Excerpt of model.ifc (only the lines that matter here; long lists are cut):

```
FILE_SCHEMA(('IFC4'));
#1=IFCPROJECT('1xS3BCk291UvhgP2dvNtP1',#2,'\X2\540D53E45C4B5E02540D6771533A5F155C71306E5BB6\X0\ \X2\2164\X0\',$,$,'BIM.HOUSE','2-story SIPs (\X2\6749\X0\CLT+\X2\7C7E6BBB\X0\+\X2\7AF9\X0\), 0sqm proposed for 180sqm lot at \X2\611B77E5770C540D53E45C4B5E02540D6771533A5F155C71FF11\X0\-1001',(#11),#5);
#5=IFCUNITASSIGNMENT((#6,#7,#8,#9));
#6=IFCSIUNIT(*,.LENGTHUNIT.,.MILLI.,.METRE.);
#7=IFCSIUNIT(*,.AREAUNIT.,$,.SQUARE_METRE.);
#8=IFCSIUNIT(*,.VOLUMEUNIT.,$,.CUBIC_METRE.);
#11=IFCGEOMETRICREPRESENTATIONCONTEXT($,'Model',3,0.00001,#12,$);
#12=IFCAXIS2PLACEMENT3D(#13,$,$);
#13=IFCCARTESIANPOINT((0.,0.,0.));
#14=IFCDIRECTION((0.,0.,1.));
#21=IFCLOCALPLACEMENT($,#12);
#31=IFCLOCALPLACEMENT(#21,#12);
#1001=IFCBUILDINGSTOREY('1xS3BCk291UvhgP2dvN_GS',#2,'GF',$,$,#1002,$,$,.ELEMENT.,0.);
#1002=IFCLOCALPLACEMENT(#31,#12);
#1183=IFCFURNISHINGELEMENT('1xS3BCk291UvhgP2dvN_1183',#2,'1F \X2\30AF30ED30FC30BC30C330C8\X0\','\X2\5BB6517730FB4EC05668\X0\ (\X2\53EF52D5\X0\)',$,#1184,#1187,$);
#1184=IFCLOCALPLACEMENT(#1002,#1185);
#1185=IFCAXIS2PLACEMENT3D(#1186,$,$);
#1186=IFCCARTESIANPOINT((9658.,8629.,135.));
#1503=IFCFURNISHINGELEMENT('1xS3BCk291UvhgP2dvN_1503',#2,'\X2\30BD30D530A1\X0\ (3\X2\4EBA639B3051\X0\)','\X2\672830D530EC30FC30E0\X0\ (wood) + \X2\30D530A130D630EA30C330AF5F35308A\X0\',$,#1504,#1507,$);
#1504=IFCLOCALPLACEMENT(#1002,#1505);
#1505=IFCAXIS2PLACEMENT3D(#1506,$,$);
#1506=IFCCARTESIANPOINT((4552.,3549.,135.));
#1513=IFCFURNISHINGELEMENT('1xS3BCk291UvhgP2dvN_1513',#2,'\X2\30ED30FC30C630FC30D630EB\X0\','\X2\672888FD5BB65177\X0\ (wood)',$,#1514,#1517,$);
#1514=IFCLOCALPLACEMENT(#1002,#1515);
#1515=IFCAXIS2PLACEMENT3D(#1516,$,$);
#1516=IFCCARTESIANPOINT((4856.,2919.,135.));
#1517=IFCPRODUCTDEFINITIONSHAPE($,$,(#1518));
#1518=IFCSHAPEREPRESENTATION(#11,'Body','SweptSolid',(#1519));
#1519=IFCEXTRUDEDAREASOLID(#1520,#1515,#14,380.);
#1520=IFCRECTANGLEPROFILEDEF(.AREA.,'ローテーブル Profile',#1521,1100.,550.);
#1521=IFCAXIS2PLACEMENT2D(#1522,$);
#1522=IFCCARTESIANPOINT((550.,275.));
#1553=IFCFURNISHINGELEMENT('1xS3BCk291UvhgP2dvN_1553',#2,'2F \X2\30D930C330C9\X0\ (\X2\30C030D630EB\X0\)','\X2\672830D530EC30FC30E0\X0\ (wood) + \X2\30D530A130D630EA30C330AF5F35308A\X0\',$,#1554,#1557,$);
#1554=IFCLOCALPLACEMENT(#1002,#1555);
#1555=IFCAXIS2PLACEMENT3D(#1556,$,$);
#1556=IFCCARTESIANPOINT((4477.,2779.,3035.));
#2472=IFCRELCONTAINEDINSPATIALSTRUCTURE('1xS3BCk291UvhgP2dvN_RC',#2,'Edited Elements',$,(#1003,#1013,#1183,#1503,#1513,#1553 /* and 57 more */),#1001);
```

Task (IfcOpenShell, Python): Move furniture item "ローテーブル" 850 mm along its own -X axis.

```python
import ifcopenshell
import ifcopenshell.api.geometry
import ifcopenshell.util.placement
import ifcopenshell.util.unit

model = ifcopenshell.open("model.ifc")
unit_scale = ifcopenshell.util.unit.calculate_unit_scale(model)

item = model.by_guid("1xS3BCk291UvhgP2dvN_1513")
matrix = ifcopenshell.util.placement.get_local_placement(item.ObjectPlacement)
matrix[:3, 3] -= matrix[:3, 0] * 0.85 / unit_scale
ifcopenshell.api.geometry.edit_object_placement(model, product=item, matrix=matrix, is_si=False)

print(ifcopenshell.util.placement.get_local_placement(item.ObjectPlacement).round(3) + 0.0)

model.write("model_rev.ifc")
```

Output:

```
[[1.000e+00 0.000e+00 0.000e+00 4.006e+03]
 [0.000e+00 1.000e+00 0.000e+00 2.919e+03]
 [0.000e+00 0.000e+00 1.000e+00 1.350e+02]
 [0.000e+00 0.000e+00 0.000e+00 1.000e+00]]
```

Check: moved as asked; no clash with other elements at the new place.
